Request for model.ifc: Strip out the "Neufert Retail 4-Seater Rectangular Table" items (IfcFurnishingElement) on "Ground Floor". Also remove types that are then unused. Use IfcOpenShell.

First a look at what the model holds.

```python
import ifcopenshell
import ifcopenshell.util.element

model = ifcopenshell.open("model.ifc")
print(model.schema)
storey = next(s for s in model.by_type("IfcBuildingStorey") if s.Name == "Ground Floor")
furniture = [e for e in ifcopenshell.util.element.get_decomposition(storey) if e.is_a("IfcFurnishingElement")]
seen = {}
for e in furniture:
    element_type = ifcopenshell.util.element.get_type(e)
    name = element_type.Name if element_type not in (None, e) else None
    seen[name] = seen.get(name, 0) + 1
for name, count in sorted(seen.items(), key=str):
    print(count, "x", name)
```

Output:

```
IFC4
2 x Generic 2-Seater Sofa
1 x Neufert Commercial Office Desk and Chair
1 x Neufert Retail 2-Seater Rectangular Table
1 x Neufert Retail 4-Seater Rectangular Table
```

```python
import ifcopenshell
import ifcopenshell.api.root
import ifcopenshell.util.element

model = ifcopenshell.open("model.ifc")

storey = next(s for s in model.by_type("IfcBuildingStorey") if s.Name == "Ground Floor")
furniture = [e for e in ifcopenshell.util.element.get_decomposition(storey) if e.is_a("IfcFurnishingElement")]
targets = [e for e in furniture if (t := ifcopenshell.util.element.get_type(e)) not in (None, e) and t.Name == "Neufert Retail 4-Seater Rectangular Table"]
types = {ifcopenshell.util.element.get_type(e) for e in targets} - {None, *targets}

for e in targets:
    ifcopenshell.api.root.remove_product(model, product=e)
print(len(targets), "removed")

unused = [t for t in types if not ifcopenshell.util.element.get_types(t)]
for t in unused:
    ifcopenshell.api.root.remove_product(model, product=t)
print(len(unused), "unused types removed")

model.write("model_edited.ifc")
```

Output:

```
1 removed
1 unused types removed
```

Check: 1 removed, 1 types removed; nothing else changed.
